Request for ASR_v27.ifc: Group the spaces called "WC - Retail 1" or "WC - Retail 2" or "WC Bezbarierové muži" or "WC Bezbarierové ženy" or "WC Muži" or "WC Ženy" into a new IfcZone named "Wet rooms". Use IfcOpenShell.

First a look at what the model holds.

```python
import ifcopenshell

model = ifcopenshell.open("ASR_v27.ifc")
print(model.schema)
seen = {}
for space in model.by_type("IfcSpace"):
    seen[space.LongName] = seen.get(space.LongName, 0) + 1
for name, count in sorted(seen.items(), key=str):
    print(count, "x", name)
print("zones:", [z.Name for z in model.by_type("IfcZone")][:20])
```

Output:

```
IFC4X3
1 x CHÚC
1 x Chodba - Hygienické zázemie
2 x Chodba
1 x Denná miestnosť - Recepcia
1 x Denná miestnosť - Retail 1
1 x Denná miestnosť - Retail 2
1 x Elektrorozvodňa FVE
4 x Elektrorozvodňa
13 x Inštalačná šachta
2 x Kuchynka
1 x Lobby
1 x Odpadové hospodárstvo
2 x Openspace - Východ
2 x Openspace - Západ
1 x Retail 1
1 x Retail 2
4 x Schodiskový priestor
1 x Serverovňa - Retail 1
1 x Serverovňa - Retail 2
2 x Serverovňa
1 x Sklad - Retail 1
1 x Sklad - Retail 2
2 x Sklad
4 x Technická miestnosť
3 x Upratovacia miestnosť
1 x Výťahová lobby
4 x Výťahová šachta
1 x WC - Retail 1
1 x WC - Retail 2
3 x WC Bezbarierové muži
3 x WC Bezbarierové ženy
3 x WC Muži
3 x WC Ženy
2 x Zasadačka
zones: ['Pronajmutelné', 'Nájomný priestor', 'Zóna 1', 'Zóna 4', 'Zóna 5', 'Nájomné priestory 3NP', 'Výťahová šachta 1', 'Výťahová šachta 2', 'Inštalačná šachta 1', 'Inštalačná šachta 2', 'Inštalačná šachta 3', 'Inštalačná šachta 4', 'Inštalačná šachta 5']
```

```python
import ifcopenshell
import ifcopenshell.api.group
import ifcopenshell.api.root

model = ifcopenshell.open("ASR_v27.ifc")

names = {"WC - Retail 1", "WC - Retail 2", "WC Bezbarierové muži", "WC Bezbarierové ženy", "WC Muži", "WC Ženy"}
spaces = [s for s in model.by_type("IfcSpace") if s.LongName in names]

zone = ifcopenshell.api.root.create_entity(model, ifc_class="IfcZone", name="Wet rooms")
ifcopenshell.api.group.assign_group(model, products=spaces, group=zone)
print(len(spaces), "spaces in", zone.Name)

model.write("ASR_v27_v2.ifc")
```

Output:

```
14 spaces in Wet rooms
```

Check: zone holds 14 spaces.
